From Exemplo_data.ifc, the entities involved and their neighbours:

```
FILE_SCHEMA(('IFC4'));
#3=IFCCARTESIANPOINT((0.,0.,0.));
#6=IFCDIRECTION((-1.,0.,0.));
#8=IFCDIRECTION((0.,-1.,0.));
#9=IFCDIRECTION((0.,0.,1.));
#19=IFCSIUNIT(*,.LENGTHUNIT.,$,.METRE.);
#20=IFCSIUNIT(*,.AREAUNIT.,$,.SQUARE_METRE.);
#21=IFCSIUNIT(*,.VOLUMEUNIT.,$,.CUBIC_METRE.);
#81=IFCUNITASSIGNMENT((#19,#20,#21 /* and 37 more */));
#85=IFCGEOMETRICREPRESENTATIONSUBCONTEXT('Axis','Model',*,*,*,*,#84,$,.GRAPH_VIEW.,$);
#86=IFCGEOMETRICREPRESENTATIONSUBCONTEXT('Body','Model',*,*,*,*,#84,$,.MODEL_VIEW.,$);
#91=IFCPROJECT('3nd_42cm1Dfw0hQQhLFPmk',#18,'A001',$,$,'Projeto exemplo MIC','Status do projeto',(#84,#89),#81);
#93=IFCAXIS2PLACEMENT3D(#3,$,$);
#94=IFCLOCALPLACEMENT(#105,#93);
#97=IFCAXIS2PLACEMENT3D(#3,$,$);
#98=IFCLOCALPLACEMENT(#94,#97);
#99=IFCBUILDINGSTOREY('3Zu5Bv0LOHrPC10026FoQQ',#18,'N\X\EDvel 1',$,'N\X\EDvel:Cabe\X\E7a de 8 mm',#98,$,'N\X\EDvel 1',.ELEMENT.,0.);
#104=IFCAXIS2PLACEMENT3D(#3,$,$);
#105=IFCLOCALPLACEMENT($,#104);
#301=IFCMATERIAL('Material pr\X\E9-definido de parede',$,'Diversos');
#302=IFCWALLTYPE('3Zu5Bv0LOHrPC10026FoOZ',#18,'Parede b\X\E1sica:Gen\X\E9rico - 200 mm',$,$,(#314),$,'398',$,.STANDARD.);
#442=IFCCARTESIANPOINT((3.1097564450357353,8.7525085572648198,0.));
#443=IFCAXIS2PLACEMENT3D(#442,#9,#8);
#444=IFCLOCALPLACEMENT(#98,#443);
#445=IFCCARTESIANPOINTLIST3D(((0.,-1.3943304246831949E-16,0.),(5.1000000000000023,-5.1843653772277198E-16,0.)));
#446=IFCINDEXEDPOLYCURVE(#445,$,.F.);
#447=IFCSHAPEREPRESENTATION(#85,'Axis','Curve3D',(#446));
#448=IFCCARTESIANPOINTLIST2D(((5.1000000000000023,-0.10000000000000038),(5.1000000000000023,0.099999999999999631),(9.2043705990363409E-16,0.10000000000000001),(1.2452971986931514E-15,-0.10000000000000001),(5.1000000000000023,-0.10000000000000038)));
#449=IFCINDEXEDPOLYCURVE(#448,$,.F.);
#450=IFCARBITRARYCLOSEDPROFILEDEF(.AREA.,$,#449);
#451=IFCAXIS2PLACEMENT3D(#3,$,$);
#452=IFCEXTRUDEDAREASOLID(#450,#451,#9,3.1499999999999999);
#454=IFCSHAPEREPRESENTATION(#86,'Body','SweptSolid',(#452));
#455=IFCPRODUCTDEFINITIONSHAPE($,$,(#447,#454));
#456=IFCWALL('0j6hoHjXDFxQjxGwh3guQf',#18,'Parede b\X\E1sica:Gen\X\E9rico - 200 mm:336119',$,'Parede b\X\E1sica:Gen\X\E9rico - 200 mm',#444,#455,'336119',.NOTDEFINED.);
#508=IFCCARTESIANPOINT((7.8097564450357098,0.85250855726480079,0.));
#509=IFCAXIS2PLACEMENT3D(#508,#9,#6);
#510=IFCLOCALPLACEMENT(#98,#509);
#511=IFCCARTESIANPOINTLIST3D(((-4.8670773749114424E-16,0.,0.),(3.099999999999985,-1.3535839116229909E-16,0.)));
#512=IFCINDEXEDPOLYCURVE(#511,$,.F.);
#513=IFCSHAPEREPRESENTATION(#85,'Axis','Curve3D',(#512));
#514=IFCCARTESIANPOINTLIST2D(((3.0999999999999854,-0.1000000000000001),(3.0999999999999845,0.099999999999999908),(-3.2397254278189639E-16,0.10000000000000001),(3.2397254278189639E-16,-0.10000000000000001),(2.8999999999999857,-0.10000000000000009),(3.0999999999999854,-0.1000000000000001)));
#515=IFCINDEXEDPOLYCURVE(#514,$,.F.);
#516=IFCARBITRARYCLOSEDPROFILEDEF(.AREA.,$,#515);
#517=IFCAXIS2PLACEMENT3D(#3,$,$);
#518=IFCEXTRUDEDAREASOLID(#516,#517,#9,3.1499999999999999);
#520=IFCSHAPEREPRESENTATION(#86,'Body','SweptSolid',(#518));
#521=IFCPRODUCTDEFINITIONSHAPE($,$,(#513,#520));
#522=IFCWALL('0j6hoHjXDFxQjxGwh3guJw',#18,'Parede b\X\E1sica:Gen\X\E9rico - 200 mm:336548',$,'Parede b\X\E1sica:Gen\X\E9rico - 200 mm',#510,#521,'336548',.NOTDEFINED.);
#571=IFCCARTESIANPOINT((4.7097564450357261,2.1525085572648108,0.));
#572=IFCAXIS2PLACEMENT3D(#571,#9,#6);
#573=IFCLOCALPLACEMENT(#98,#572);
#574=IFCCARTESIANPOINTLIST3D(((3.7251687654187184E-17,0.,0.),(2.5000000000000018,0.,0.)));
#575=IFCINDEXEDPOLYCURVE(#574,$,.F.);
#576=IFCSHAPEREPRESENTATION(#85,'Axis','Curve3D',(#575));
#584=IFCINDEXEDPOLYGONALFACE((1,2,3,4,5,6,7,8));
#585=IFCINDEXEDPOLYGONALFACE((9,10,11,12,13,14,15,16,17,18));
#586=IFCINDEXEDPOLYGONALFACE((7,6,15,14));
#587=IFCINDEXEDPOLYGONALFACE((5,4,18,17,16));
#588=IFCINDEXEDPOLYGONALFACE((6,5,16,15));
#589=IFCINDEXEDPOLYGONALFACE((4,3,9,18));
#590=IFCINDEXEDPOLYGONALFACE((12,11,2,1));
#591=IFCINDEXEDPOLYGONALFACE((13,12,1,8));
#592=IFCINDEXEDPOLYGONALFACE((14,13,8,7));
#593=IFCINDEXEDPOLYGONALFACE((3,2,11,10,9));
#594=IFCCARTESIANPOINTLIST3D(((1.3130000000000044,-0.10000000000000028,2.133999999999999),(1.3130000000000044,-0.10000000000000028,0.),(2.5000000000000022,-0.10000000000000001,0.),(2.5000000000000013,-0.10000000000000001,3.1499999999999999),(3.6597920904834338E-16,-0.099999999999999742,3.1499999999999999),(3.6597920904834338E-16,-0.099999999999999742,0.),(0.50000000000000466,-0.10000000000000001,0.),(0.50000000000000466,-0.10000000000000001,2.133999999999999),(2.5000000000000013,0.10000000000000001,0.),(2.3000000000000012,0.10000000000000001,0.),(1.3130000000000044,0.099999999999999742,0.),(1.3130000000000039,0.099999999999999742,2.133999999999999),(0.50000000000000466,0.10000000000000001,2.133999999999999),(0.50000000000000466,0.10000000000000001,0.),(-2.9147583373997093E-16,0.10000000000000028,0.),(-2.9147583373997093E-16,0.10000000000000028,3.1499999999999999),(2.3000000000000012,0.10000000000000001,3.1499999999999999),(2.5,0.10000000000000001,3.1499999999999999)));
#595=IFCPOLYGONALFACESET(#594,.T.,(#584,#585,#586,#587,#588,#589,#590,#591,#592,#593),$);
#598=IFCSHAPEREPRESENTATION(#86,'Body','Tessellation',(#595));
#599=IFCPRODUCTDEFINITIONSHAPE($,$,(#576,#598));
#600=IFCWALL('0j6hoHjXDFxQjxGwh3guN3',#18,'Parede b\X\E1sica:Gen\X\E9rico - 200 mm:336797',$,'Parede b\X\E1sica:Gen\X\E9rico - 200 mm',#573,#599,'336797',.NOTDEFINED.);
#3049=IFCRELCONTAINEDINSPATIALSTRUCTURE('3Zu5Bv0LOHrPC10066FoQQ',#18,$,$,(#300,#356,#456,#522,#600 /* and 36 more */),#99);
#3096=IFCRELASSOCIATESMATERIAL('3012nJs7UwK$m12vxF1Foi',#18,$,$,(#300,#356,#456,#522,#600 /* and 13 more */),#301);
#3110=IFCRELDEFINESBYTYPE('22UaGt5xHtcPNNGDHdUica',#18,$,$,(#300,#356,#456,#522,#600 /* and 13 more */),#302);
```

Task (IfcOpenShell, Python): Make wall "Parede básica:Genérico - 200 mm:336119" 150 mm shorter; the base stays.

```python
import ifcopenshell
import ifcopenshell.geom
import ifcopenshell.util.representation
import ifcopenshell.util.shape
import ifcopenshell.util.unit

model = ifcopenshell.open("Exemplo_data.ifc")
unit_scale = ifcopenshell.util.unit.calculate_unit_scale(model)
settings = ifcopenshell.geom.settings()


def volume(element):
    """Net volume in cubic metres, openings subtracted."""
    shape = ifcopenshell.geom.create_shape(settings, element)
    return ifcopenshell.util.shape.get_volume(shape.geometry)


wall = model.by_guid("0j6hoHjXDFxQjxGwh3guQf")
before = volume(wall)

body = ifcopenshell.util.representation.get_representation(wall, "Model", "Body")
solid = body.Items[0]
old_height = solid.Depth
solid.Depth -= 0.15 / unit_scale
after = volume(wall)

print(f"height {old_height:g} -> {solid.Depth:g}, volume {before:.3f} -> {after:.3f} m3")

model.write("Exemplo_data_edited.ifc")
```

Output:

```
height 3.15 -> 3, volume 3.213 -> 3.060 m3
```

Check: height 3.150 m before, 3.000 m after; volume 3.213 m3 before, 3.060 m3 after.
